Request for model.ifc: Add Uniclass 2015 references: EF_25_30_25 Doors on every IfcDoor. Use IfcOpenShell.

First a look at what the model holds.

```python
import ifcopenshell

model = ifcopenshell.open("model.ifc")
print(model.schema)
print("classifications:", [c.Name for c in model.by_type("IfcClassification")])
for ifc_class in ("IfcDoor", "IfcRoof", "IfcStair", "IfcWall", "IfcWindow"):
    print(ifc_class, len(model.by_type(ifc_class)))
```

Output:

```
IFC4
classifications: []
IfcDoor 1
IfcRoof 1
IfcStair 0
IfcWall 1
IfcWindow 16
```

```python
import ifcopenshell
import ifcopenshell.api.classification

model = ifcopenshell.open("model.ifc")

system = ifcopenshell.api.classification.add_classification(model, classification="Uniclass 2015")

codes = {
    "IfcDoor": ("EF_25_30_25", "Doors"),
}
for ifc_class, (code, name) in codes.items():
    products = model.by_type(ifc_class)
    ifcopenshell.api.classification.add_reference(
        model, products=products, classification=system, identification=code, name=name
    )
    print(code, len(products))

model.write("model_updated.ifc")
```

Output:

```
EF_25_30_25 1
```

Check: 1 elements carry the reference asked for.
